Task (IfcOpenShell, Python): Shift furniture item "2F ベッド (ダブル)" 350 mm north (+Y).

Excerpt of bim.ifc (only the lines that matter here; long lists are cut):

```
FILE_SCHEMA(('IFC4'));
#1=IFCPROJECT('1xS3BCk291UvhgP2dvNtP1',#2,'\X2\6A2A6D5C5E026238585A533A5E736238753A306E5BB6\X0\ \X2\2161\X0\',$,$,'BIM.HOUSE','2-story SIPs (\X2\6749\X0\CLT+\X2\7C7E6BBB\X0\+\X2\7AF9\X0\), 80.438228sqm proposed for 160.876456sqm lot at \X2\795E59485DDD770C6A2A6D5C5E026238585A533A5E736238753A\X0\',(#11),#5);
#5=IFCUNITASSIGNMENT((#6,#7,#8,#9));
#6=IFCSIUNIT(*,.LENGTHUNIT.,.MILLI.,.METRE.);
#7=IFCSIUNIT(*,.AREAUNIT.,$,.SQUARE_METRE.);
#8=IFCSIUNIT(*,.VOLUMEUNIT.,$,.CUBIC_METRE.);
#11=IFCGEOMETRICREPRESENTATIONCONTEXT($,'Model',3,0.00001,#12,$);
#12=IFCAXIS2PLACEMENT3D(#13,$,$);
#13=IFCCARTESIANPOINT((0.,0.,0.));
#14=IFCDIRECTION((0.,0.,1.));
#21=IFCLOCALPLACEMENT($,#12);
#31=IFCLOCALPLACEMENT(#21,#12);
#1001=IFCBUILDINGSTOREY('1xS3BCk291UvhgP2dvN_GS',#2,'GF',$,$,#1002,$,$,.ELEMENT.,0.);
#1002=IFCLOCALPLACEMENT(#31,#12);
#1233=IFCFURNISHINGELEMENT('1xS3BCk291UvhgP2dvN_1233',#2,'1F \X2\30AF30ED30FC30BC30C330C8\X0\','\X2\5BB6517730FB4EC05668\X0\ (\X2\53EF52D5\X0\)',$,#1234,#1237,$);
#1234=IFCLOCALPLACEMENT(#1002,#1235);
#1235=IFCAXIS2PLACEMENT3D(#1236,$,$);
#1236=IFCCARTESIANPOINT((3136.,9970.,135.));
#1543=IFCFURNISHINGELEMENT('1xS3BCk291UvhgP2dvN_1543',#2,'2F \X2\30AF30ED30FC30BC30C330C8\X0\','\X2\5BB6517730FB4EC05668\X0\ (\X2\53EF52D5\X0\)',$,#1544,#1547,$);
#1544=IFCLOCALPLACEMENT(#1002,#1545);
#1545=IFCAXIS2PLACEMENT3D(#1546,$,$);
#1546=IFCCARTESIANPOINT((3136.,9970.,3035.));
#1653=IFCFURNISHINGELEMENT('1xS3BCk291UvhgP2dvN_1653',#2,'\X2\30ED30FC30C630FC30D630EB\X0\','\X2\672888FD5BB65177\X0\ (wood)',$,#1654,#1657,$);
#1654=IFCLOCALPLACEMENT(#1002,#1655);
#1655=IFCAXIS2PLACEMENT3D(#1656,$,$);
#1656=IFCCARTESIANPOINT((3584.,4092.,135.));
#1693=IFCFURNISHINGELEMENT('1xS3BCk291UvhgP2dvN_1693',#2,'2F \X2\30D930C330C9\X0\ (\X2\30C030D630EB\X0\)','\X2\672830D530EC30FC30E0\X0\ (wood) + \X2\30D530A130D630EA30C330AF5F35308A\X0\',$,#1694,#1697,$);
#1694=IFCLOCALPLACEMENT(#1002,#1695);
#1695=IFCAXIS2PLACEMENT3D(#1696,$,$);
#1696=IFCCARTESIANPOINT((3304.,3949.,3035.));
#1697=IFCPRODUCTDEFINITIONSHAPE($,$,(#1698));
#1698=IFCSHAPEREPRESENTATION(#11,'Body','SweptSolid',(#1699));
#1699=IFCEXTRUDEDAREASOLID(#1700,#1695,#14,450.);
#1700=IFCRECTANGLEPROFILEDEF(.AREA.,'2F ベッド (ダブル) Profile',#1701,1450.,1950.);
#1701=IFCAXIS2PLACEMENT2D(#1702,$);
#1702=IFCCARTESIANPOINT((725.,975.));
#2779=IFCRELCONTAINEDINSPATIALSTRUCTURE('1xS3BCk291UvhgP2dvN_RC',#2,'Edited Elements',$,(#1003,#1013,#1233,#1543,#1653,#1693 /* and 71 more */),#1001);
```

```python
import ifcopenshell
import ifcopenshell.api.geometry
import ifcopenshell.util.placement
import ifcopenshell.util.unit

model = ifcopenshell.open("bim.ifc")
unit_scale = ifcopenshell.util.unit.calculate_unit_scale(model)

item = model.by_guid("1xS3BCk291UvhgP2dvN_1693")
matrix = ifcopenshell.util.placement.get_local_placement(item.ObjectPlacement)
matrix[1, 3] += 0.35 / unit_scale
ifcopenshell.api.geometry.edit_object_placement(model, product=item, matrix=matrix, is_si=False)

print(ifcopenshell.util.placement.get_local_placement(item.ObjectPlacement).round(3) + 0.0)

model.write("bim-out.ifc")
```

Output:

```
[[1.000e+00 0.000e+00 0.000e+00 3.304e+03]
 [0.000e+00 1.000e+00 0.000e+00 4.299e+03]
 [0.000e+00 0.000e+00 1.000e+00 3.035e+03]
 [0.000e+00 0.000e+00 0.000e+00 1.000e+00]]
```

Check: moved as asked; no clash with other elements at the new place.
